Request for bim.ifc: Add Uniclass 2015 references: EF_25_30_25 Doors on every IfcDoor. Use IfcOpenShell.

First a look at what the model holds.

```python
import ifcopenshell

model = ifcopenshell.open("bim.ifc")
print(model.schema)
print("classifications:", [c.Name for c in model.by_type("IfcClassification")])
for ifc_class in ("IfcDoor", "IfcRoof", "IfcStair", "IfcWall", "IfcWindow"):
    print(ifc_class, len(model.by_type(ifc_class)))
```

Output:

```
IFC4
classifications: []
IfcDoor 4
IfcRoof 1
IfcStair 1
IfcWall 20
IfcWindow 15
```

```python
import ifcopenshell
import ifcopenshell.api.classification

model = ifcopenshell.open("bim.ifc")

system = ifcopenshell.api.classification.add_classification(model, classification="Uniclass 2015")

codes = {
    "IfcDoor": ("EF_25_30_25", "Doors"),
}
for ifc_class, (code, name) in codes.items():
    products = model.by_type(ifc_class)
    ifcopenshell.api.classification.add_reference(
        model, products=products, classification=system, identification=code, name=name
    )
    print(code, len(products))

model.write("bim-out.ifc")
```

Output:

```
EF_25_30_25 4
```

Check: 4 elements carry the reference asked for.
